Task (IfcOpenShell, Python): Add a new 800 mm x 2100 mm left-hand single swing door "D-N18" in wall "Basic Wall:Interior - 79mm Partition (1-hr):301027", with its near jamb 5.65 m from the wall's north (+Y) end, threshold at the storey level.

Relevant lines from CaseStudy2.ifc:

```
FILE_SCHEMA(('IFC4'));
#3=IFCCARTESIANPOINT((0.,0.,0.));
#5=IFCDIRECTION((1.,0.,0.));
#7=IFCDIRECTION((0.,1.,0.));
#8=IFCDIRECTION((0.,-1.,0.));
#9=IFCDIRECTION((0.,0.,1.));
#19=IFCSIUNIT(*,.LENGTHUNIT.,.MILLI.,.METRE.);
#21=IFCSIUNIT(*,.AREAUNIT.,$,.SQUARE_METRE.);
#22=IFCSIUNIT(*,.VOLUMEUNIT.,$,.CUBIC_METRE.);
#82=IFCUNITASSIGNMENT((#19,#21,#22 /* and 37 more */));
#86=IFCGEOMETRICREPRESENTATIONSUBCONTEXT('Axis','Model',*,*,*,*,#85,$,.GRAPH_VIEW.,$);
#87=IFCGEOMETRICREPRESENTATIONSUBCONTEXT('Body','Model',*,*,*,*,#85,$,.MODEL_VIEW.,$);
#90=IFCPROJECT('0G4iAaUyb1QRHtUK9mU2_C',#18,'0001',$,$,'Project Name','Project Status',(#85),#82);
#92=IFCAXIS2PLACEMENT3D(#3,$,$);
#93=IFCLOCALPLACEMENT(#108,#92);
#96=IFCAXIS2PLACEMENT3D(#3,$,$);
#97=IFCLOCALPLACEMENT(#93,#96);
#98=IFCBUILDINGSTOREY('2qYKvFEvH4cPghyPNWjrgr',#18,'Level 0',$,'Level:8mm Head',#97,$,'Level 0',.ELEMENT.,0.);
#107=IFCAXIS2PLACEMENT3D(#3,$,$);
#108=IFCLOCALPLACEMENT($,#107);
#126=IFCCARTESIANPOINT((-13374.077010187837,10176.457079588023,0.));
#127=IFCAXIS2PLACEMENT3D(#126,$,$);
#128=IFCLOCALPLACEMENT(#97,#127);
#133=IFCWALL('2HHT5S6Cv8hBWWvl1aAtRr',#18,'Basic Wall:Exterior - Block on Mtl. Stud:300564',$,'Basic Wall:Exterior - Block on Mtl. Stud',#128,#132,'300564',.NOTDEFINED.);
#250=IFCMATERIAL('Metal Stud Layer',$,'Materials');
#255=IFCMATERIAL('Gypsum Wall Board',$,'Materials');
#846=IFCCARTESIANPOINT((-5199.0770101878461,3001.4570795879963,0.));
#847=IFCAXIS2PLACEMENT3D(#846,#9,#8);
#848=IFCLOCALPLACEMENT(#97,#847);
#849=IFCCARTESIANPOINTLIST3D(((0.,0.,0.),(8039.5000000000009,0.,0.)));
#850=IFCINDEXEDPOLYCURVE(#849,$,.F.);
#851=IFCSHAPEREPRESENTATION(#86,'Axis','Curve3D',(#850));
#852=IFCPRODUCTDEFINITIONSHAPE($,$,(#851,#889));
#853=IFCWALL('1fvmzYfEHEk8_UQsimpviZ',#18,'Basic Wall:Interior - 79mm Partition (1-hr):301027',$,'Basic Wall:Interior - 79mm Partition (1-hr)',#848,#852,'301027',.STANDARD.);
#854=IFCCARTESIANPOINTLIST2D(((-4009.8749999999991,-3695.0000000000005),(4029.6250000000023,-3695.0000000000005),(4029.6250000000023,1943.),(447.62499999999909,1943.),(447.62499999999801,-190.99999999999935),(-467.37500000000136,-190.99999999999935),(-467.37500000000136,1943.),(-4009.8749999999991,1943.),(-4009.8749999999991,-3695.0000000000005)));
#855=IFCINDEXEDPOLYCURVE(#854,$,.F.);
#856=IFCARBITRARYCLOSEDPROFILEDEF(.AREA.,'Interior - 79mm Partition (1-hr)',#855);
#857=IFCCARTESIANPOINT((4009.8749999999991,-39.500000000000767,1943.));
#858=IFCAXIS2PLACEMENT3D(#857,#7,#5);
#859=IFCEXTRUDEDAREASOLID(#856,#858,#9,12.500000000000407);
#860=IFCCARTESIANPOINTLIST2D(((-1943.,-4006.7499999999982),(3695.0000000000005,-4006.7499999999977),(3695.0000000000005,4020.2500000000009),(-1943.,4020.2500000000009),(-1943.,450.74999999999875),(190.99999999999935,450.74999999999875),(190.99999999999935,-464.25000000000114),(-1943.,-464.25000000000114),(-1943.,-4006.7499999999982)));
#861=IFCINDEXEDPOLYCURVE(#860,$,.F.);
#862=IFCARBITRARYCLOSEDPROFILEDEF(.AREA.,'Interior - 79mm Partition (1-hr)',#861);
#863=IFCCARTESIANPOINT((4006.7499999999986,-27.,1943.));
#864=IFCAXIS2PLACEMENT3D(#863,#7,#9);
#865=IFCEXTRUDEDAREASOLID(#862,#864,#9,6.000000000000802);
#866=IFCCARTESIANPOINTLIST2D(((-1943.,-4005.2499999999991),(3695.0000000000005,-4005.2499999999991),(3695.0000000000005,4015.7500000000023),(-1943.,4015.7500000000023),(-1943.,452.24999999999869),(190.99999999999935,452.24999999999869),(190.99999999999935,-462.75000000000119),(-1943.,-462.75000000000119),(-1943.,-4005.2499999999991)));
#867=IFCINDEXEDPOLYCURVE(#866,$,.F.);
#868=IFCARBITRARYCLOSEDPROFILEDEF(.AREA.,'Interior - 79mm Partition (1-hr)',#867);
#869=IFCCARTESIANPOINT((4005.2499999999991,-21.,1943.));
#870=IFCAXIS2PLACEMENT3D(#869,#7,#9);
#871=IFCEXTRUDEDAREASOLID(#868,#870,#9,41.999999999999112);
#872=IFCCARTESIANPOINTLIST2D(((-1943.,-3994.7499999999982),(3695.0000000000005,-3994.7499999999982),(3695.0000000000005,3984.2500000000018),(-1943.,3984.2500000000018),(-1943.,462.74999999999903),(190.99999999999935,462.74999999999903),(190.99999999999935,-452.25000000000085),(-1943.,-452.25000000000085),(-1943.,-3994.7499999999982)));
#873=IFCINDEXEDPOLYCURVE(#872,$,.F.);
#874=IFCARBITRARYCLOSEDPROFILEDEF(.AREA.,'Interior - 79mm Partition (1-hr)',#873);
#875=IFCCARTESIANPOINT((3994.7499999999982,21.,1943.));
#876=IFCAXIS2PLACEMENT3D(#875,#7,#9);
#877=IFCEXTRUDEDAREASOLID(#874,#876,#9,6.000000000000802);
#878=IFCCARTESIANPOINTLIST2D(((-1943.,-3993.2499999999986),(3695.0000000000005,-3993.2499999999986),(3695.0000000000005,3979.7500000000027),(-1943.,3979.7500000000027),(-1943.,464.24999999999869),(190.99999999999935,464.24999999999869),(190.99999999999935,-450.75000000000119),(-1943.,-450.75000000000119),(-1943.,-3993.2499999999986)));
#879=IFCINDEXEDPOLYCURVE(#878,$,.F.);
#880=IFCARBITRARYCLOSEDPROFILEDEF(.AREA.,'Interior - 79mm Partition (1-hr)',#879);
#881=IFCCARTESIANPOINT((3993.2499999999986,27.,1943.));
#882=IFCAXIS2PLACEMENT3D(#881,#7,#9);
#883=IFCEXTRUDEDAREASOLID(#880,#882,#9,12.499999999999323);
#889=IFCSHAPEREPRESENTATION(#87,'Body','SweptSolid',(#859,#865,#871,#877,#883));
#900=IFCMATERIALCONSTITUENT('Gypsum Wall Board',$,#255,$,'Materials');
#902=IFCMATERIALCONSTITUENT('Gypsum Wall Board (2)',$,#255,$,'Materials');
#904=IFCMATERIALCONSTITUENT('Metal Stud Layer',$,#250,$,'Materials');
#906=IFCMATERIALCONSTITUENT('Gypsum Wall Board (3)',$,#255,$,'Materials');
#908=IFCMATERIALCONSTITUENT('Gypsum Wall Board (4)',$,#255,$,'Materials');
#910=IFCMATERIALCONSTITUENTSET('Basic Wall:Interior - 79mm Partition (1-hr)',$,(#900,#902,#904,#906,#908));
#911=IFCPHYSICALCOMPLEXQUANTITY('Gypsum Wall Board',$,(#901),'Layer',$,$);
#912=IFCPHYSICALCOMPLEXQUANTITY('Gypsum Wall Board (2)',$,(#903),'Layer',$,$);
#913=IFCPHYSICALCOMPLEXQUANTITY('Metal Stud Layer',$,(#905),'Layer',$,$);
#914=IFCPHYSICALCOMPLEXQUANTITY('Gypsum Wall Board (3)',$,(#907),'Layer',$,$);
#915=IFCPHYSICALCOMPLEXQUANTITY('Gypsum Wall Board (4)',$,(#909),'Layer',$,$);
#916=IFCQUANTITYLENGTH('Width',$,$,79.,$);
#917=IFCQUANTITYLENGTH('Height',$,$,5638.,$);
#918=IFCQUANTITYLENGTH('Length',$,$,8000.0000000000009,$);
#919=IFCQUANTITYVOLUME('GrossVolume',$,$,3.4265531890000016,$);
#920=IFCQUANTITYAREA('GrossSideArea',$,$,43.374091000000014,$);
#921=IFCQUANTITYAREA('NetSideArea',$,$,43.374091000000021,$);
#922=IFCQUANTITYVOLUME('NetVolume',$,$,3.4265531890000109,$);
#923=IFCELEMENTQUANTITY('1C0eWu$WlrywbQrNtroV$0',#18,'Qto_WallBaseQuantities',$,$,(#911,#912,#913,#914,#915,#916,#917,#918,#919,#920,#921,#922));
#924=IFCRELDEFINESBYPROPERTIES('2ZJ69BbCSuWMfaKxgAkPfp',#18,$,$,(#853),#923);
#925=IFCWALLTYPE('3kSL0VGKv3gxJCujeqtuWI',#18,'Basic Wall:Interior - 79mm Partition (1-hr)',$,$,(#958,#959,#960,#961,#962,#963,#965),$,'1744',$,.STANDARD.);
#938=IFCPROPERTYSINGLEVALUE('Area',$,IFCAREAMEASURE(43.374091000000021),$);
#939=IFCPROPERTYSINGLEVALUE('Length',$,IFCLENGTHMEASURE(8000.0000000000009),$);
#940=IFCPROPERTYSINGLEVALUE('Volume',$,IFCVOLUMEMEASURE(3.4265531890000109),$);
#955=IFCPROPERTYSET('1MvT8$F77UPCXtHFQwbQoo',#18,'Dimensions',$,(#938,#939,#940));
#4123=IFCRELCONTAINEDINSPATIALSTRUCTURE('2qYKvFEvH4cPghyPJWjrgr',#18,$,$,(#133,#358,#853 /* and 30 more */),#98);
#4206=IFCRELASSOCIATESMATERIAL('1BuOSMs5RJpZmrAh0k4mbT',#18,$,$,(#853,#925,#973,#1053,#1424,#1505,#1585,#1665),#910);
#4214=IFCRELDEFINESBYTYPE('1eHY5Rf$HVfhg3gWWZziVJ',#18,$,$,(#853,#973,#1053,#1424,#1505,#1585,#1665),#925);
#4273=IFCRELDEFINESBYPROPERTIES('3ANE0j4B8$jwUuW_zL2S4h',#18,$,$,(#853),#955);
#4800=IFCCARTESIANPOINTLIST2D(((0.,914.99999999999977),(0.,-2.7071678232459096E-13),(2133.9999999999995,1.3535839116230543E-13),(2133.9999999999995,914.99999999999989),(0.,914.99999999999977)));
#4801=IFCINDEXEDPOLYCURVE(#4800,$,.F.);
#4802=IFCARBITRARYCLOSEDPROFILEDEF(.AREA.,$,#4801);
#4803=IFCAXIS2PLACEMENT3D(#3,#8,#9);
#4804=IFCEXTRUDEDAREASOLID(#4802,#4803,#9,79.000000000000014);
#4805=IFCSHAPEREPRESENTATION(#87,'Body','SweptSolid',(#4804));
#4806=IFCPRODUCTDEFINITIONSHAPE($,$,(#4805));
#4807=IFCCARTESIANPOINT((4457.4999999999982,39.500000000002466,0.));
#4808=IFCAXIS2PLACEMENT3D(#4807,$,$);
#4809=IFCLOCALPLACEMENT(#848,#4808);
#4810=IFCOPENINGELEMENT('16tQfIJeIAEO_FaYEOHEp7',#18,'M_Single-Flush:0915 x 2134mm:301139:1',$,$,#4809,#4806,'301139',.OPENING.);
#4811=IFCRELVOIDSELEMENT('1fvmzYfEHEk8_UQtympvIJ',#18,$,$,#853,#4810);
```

```python
import numpy as np
import ifcopenshell
import ifcopenshell.api.feature
import ifcopenshell.api.geometry
import ifcopenshell.api.pset
import ifcopenshell.api.root
import ifcopenshell.api.spatial
import ifcopenshell.geom
import ifcopenshell.util.element
import ifcopenshell.util.placement
import ifcopenshell.util.representation
import ifcopenshell.util.shape
import ifcopenshell.util.unit

model = ifcopenshell.open("CaseStudy2.ifc")
unit_scale = ifcopenshell.util.unit.calculate_unit_scale(model)
area_scale = ifcopenshell.util.unit.calculate_unit_scale(model, "AREAUNIT")
volume_scale = ifcopenshell.util.unit.calculate_unit_scale(model, "VOLUMEUNIT")
settings = ifcopenshell.geom.settings()


def volume(element):
    """Net volume in cubic metres, openings subtracted."""
    shape = ifcopenshell.geom.create_shape(settings, element)
    return ifcopenshell.util.shape.get_volume(shape.geometry)


wall = model.by_guid("1fvmzYfEHEk8_UQsimpviZ")
storey = ifcopenshell.util.element.get_container(wall, ifc_class="IfcBuildingStorey")
context = ifcopenshell.util.representation.get_context(model, "Model", "Body", "MODEL_VIEW")
before = volume(wall)

width, height, from_end, sill = 0.8, 2.1, 5.65, 0.0  # metres

# The wall runs along its own X axis, and the end named is its -X end.
wall_shape = ifcopenshell.geom.create_shape(settings, wall)
x, y, z = ifcopenshell.util.shape.get_vertices(wall_shape.geometry).T
start = x.min() + from_end
face, thickness = float(y.min()), float(y.max() - y.min())
wall_matrix = ifcopenshell.util.placement.get_local_placement(wall.ObjectPlacement)
level = ifcopenshell.util.placement.get_local_placement(storey.ObjectPlacement)[2, 3]


def in_wall(x, y):
    """Placement at x, y metres in the wall's axes, at sill height."""
    matrix = wall_matrix.copy()
    matrix[:, 3] = wall_matrix @ np.array([x / unit_scale, y / unit_scale, 0.0, 1.0])
    matrix[2, 3] = level + sill / unit_scale
    return matrix


# Opening: a box that overshoots both wall faces by 50 mm.
opening = ifcopenshell.api.root.create_entity(model, ifc_class="IfcOpeningElement", predefined_type="OPENING")
box = ifcopenshell.api.geometry.add_wall_representation(
    model, context=context, length=width, height=height, thickness=thickness + 0.1
)
ifcopenshell.api.geometry.assign_representation(model, product=opening, representation=box)
ifcopenshell.api.geometry.edit_object_placement(model, product=opening, matrix=in_wall(start, face - 0.05), is_si=False)
ifcopenshell.api.feature.add_feature(model, feature=opening, element=wall)

door = ifcopenshell.api.root.create_entity(model, ifc_class="IfcDoor", name="D-N18", predefined_type="DOOR")
door.OverallWidth, door.OverallHeight = width / unit_scale, height / unit_scale
door.OperationType = "SINGLE_SWING_LEFT"
body = ifcopenshell.api.geometry.add_door_representation(
    model,
    context=context,
    overall_width=door.OverallWidth,
    overall_height=door.OverallHeight,
    operation_type="SINGLE_SWING_LEFT",
    lining_properties={"LiningDepth": thickness / unit_scale, "ThresholdDepth": thickness / unit_scale},
)
ifcopenshell.api.geometry.assign_representation(model, product=door, representation=body)
ifcopenshell.api.spatial.assign_container(model, products=[door], relating_structure=storey)
ifcopenshell.api.feature.add_filling(model, opening=opening, element=door)

# The lining spans the wall, so the door starts at the wall face.
ifcopenshell.api.geometry.edit_object_placement(model, product=door, matrix=in_wall(start, face), is_si=False)

after = volume(wall)

# Update the wall's stored quantities.
qto = model.by_id(ifcopenshell.util.element.get_pset(wall, "Qto_WallBaseQuantities", should_inherit=False)["id"])
ifcopenshell.api.pset.edit_qto(model, qto=qto, properties={
    "NetSideArea": after / thickness / area_scale,
    "NetVolume": after / volume_scale,
})
pset = model.by_id(ifcopenshell.util.element.get_pset(wall, "Dimensions", should_inherit=False)["id"])
ifcopenshell.api.pset.edit_pset(model, pset=pset, properties={
    "Area": model.create_entity("IfcAreaMeasure", after / thickness / area_scale),
    "Volume": model.create_entity("IfcVolumeMeasure", after / volume_scale),
})

print(f"wall volume {before:.3f} -> {after:.3f} m3")

model.write("CaseStudy2-out.ifc")
```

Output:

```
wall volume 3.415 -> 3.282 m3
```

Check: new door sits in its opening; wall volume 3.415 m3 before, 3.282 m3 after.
